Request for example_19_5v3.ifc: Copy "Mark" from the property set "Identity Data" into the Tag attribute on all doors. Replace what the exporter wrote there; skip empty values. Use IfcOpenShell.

First a look at what the model holds.

```python
import ifcopenshell
import ifcopenshell.util.element

model = ifcopenshell.open("example_19_5v3.ifc")
print(model.schema)
doors = model.by_type("IfcDoor")
print(len(doors), "doors")
for e in doors[:8]:
    source = ifcopenshell.util.element.get_pset(e, "Identity Data", "Mark")
    target = e.Tag
    print(e.id(), repr(source), repr(target), sep=" | ")
```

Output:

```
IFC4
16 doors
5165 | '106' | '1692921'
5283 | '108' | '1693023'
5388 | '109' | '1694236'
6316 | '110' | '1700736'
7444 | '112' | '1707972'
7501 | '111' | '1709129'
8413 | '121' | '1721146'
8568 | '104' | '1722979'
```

```python
import ifcopenshell
import ifcopenshell.util.element

model = ifcopenshell.open("example_19_5v3.ifc")

count = 0
for e in model.by_type("IfcDoor"):
    value = ifcopenshell.util.element.get_pset(e, "Identity Data", "Mark")
    current = e.Tag
    if not value or not value.strip() or current == value:
        continue
    e.Tag = value
    count += 1

print(count, "doors updated")

model.write("example_19_5v3_v2.ifc")
```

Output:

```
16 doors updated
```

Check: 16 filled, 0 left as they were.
